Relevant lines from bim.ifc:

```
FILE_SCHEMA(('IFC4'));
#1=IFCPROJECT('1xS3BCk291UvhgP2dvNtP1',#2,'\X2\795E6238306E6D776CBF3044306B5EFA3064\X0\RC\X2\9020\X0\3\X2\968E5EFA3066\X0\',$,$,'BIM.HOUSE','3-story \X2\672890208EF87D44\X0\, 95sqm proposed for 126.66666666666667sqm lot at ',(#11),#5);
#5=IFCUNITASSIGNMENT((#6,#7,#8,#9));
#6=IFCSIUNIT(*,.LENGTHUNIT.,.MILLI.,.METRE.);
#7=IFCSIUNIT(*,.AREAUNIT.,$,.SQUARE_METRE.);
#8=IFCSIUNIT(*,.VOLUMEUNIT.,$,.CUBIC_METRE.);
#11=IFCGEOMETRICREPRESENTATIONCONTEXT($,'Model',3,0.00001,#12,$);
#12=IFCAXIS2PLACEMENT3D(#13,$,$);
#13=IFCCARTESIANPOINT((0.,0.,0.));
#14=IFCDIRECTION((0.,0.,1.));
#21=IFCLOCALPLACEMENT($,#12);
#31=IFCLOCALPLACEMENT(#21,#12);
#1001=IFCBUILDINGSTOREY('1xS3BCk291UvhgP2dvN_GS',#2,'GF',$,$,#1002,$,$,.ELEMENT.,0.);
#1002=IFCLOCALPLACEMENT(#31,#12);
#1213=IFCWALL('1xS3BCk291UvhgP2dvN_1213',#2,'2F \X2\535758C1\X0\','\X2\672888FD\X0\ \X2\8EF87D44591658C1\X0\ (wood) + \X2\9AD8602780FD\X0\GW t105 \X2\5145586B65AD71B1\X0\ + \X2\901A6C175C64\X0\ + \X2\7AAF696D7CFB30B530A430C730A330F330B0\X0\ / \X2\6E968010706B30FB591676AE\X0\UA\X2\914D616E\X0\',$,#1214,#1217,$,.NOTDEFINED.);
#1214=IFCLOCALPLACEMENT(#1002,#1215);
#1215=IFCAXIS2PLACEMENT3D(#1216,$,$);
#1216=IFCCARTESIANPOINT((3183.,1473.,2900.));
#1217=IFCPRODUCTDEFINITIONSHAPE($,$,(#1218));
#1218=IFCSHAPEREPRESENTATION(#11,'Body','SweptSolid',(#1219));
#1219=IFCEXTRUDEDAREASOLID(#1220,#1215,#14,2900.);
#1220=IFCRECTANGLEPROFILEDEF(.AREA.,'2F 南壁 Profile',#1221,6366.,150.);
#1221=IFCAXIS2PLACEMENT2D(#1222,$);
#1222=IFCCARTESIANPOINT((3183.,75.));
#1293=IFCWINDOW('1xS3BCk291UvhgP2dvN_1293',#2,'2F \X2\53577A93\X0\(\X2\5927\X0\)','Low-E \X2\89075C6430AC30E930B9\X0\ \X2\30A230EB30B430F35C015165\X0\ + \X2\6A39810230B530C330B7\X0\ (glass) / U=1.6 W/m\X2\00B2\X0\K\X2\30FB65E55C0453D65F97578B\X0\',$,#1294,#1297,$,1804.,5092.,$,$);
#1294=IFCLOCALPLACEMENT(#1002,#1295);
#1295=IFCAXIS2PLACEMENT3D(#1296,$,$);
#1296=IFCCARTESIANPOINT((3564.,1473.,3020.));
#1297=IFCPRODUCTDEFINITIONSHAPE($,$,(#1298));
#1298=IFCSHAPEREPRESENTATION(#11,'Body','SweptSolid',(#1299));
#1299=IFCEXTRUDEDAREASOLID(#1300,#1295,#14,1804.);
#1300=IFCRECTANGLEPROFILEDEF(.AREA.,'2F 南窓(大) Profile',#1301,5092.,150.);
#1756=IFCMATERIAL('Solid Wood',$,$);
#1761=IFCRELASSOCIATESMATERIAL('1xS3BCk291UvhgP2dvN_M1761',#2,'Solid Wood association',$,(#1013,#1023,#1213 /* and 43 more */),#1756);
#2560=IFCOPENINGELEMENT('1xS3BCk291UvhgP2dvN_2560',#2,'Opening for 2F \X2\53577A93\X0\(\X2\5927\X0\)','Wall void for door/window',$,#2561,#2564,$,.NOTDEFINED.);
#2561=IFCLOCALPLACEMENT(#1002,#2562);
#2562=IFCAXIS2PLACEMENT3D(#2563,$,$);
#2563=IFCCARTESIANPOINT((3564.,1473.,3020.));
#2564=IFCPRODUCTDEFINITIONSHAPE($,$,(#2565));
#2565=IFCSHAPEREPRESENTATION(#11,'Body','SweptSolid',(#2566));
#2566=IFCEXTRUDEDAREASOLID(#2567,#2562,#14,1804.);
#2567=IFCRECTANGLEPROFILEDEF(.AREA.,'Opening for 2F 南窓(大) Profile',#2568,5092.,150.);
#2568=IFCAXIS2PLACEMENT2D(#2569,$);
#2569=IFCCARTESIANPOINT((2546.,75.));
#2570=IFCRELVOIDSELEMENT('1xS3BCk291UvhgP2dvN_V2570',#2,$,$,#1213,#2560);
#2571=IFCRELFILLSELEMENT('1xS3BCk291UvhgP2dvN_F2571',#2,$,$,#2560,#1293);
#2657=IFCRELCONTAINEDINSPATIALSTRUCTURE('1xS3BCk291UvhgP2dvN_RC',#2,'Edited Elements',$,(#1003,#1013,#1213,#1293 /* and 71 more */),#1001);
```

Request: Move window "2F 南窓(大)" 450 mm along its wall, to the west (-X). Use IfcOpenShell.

```python
import ifcopenshell
import ifcopenshell.api.geometry
import ifcopenshell.util.placement
import ifcopenshell.util.unit

model = ifcopenshell.open("bim.ifc")
unit_scale = ifcopenshell.util.unit.calculate_unit_scale(model)

window = model.by_guid("1xS3BCk291UvhgP2dvN_1293")
opening = window.FillsVoids[0].RelatingOpeningElement
wall = opening.VoidsElements[0].RelatingBuildingElement

wall_matrix = ifcopenshell.util.placement.get_local_placement(wall.ObjectPlacement)
shift = wall_matrix[:3, 0] * -0.45 / unit_scale
before = ifcopenshell.util.placement.get_local_placement(window.ObjectPlacement)[:3, 3].copy()

# The window is not placed relative to its opening, so move both.
for product in (opening, window):
    matrix = ifcopenshell.util.placement.get_local_placement(product.ObjectPlacement)
    matrix[:3, 3] += shift
    ifcopenshell.api.geometry.edit_object_placement(model, product=product, matrix=matrix, is_si=False)

after = ifcopenshell.util.placement.get_local_placement(window.ObjectPlacement)[:3, 3]
print("window moved by", (after - before).round(3) + 0.0)

model.write("bim-out.ifc")
```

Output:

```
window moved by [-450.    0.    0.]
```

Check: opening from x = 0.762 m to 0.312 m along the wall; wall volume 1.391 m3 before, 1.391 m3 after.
